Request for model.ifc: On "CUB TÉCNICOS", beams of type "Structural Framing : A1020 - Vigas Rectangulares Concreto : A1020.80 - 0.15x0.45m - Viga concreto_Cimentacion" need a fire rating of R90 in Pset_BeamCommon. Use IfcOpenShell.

First a look at what the model holds.

```python
import ifcopenshell
import ifcopenshell.util.element

model = ifcopenshell.open("model.ifc")
print(model.schema)
storey = next(s for s in model.by_type("IfcBuildingStorey") if s.Name == "CUB TÉCNICOS")
beams = [e for e in ifcopenshell.util.element.get_decomposition(storey) if e.is_a("IfcBeam")]
seen = {}
for e in beams:
    element_type = ifcopenshell.util.element.get_type(e)
    key = (element_type.Name if element_type != e and element_type else None, ifcopenshell.util.element.get_pset(e, "Pset_BeamCommon", "FireRating"))
    seen[key] = seen.get(key, 0) + 1
for (name, value), count in sorted(seen.items(), key=str):
    print(count, "x", name, "|", value)
```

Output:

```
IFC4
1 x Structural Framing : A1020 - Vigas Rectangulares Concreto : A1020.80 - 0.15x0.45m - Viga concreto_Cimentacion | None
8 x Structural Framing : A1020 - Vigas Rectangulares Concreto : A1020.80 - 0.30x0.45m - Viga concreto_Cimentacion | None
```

```python
import ifcopenshell
import ifcopenshell.api.pset
import ifcopenshell.util.element

model = ifcopenshell.open("model.ifc")

storey = next(s for s in model.by_type("IfcBuildingStorey") if s.Name == "CUB TÉCNICOS")
beams = [e for e in ifcopenshell.util.element.get_decomposition(storey) if e.is_a("IfcBeam")]

count = 0
for e in beams:
    element_type = ifcopenshell.util.element.get_type(e)
    if element_type in (None, e) or element_type.Name != "Structural Framing : A1020 - Vigas Rectangulares Concreto : A1020.80 - 0.15x0.45m - Viga concreto_Cimentacion":
        continue
    # add_pset returns the element's existing set when there is one.
    pset = ifcopenshell.api.pset.add_pset(model, product=e, name="Pset_BeamCommon")
    ifcopenshell.api.pset.edit_pset(model, pset=pset, properties={"FireRating": "R90"})
    count += 1

print(count, "beams updated")

model.write("model_edited.ifc")
```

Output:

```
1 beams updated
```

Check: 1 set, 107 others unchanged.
